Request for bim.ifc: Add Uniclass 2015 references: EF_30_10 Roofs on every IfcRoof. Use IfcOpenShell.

First a look at what the model holds.

```python
import ifcopenshell

model = ifcopenshell.open("bim.ifc")
print(model.schema)
print("classifications:", [c.Name for c in model.by_type("IfcClassification")])
for ifc_class in ("IfcDoor", "IfcRoof", "IfcStair", "IfcWall", "IfcWindow"):
    print(ifc_class, len(model.by_type(ifc_class)))
```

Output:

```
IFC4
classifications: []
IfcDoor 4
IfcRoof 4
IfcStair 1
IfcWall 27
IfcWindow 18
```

```python
import ifcopenshell
import ifcopenshell.api.classification

model = ifcopenshell.open("bim.ifc")

system = ifcopenshell.api.classification.add_classification(model, classification="Uniclass 2015")

codes = {
    "IfcRoof": ("EF_30_10", "Roofs"),
}
for ifc_class, (code, name) in codes.items():
    products = model.by_type(ifc_class)
    ifcopenshell.api.classification.add_reference(
        model, products=products, classification=system, identification=code, name=name
    )
    print(code, len(products))

model.write("bim-out.ifc")
```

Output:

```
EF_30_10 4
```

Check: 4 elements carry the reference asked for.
